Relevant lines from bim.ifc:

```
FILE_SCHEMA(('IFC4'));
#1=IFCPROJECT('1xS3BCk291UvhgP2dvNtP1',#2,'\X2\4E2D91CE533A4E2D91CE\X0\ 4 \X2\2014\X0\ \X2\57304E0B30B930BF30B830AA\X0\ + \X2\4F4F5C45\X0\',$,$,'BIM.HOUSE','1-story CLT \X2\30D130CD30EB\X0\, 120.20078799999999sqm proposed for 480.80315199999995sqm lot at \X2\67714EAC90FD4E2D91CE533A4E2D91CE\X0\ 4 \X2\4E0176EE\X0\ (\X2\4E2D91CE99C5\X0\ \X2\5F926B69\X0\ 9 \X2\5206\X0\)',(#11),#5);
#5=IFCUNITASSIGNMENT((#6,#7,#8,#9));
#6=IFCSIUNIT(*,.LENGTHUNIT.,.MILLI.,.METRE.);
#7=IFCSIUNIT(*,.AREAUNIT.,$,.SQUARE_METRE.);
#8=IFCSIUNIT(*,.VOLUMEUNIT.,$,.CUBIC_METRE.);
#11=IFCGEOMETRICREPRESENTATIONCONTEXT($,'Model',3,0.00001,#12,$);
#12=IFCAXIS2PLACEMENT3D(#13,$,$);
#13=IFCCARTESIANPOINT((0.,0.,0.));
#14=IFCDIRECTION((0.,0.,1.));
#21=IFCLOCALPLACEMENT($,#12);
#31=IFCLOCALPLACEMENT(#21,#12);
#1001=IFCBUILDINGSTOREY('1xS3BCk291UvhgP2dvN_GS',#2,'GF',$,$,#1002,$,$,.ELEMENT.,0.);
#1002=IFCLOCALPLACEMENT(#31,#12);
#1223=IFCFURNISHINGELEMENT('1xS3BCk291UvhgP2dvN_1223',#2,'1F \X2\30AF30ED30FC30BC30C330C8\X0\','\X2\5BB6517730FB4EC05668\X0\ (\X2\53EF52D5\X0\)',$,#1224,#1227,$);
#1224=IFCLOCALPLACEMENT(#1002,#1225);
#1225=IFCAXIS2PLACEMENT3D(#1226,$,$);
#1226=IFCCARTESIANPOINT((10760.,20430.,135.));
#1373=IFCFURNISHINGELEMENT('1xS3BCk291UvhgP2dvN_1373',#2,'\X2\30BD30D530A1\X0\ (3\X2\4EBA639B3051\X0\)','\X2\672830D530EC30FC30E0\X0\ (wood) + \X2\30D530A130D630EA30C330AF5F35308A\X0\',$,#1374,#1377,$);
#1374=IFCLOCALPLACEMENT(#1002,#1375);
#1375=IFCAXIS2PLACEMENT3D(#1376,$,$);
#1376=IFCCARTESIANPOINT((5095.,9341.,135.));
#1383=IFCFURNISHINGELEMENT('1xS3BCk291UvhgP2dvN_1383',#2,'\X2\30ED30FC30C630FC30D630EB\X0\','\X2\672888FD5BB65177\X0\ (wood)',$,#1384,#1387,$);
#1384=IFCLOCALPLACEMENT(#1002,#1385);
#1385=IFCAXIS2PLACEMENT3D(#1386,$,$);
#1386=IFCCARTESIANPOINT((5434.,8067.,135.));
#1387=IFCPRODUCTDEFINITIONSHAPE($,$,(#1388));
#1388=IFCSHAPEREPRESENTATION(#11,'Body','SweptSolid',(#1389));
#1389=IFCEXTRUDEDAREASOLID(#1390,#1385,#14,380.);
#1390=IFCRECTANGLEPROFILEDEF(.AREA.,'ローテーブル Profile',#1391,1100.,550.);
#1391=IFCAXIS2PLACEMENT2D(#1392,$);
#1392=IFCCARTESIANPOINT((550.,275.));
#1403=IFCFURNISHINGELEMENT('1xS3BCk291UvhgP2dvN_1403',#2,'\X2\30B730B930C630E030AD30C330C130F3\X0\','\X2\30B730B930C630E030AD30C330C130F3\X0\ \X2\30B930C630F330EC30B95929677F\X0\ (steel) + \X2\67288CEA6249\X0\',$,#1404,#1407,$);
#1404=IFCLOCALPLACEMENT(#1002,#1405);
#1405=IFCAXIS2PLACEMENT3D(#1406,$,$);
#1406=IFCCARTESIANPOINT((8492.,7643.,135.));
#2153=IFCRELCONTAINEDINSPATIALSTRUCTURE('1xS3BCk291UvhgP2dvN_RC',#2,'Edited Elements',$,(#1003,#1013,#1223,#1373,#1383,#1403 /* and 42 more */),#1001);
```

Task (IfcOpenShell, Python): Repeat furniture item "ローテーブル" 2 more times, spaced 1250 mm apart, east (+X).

```python
import numpy as np
import ifcopenshell
import ifcopenshell.api.geometry
import ifcopenshell.api.root
import ifcopenshell.util.element
import ifcopenshell.util.placement
import ifcopenshell.util.unit

model = ifcopenshell.open("bim.ifc")
unit_scale = ifcopenshell.util.unit.calculate_unit_scale(model)


def reuse_history(source, copy):
    """copy_class also copies each property set's owner history, people and application; keep the originals."""
    for rel in copy.IsDefinedBy:
        if rel.is_a("IfcRelDefinesByProperties") and (history := rel.RelatingPropertyDefinition.OwnerHistory):
            rel.RelatingPropertyDefinition.OwnerHistory = source.OwnerHistory
            ifcopenshell.util.element.remove_deep2(model, history)


source = model.by_id(1383)
base = ifcopenshell.util.placement.get_local_placement(source.ObjectPlacement)
step = np.array([1.0, 0.0, 0.0]) * 1.25 / unit_scale

for i in range(1, 3):
    copy = ifcopenshell.api.root.copy_class(model, product=source)
    copy.Representation = ifcopenshell.util.element.copy_deep(
        model, source.Representation, exclude=["IfcGeometricRepresentationContext", "IfcRepresentationMap"]
    )
    reuse_history(source, copy)
    matrix = base.copy()
    matrix[:3, 3] += i * step
    print("added at", matrix[:3, 3].round(3) + 0.0)
    ifcopenshell.api.geometry.edit_object_placement(model, product=copy, matrix=matrix, is_si=False)

model.write("bim_rev.ifc")
```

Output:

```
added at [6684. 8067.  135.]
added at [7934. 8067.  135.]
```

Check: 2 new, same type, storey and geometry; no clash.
